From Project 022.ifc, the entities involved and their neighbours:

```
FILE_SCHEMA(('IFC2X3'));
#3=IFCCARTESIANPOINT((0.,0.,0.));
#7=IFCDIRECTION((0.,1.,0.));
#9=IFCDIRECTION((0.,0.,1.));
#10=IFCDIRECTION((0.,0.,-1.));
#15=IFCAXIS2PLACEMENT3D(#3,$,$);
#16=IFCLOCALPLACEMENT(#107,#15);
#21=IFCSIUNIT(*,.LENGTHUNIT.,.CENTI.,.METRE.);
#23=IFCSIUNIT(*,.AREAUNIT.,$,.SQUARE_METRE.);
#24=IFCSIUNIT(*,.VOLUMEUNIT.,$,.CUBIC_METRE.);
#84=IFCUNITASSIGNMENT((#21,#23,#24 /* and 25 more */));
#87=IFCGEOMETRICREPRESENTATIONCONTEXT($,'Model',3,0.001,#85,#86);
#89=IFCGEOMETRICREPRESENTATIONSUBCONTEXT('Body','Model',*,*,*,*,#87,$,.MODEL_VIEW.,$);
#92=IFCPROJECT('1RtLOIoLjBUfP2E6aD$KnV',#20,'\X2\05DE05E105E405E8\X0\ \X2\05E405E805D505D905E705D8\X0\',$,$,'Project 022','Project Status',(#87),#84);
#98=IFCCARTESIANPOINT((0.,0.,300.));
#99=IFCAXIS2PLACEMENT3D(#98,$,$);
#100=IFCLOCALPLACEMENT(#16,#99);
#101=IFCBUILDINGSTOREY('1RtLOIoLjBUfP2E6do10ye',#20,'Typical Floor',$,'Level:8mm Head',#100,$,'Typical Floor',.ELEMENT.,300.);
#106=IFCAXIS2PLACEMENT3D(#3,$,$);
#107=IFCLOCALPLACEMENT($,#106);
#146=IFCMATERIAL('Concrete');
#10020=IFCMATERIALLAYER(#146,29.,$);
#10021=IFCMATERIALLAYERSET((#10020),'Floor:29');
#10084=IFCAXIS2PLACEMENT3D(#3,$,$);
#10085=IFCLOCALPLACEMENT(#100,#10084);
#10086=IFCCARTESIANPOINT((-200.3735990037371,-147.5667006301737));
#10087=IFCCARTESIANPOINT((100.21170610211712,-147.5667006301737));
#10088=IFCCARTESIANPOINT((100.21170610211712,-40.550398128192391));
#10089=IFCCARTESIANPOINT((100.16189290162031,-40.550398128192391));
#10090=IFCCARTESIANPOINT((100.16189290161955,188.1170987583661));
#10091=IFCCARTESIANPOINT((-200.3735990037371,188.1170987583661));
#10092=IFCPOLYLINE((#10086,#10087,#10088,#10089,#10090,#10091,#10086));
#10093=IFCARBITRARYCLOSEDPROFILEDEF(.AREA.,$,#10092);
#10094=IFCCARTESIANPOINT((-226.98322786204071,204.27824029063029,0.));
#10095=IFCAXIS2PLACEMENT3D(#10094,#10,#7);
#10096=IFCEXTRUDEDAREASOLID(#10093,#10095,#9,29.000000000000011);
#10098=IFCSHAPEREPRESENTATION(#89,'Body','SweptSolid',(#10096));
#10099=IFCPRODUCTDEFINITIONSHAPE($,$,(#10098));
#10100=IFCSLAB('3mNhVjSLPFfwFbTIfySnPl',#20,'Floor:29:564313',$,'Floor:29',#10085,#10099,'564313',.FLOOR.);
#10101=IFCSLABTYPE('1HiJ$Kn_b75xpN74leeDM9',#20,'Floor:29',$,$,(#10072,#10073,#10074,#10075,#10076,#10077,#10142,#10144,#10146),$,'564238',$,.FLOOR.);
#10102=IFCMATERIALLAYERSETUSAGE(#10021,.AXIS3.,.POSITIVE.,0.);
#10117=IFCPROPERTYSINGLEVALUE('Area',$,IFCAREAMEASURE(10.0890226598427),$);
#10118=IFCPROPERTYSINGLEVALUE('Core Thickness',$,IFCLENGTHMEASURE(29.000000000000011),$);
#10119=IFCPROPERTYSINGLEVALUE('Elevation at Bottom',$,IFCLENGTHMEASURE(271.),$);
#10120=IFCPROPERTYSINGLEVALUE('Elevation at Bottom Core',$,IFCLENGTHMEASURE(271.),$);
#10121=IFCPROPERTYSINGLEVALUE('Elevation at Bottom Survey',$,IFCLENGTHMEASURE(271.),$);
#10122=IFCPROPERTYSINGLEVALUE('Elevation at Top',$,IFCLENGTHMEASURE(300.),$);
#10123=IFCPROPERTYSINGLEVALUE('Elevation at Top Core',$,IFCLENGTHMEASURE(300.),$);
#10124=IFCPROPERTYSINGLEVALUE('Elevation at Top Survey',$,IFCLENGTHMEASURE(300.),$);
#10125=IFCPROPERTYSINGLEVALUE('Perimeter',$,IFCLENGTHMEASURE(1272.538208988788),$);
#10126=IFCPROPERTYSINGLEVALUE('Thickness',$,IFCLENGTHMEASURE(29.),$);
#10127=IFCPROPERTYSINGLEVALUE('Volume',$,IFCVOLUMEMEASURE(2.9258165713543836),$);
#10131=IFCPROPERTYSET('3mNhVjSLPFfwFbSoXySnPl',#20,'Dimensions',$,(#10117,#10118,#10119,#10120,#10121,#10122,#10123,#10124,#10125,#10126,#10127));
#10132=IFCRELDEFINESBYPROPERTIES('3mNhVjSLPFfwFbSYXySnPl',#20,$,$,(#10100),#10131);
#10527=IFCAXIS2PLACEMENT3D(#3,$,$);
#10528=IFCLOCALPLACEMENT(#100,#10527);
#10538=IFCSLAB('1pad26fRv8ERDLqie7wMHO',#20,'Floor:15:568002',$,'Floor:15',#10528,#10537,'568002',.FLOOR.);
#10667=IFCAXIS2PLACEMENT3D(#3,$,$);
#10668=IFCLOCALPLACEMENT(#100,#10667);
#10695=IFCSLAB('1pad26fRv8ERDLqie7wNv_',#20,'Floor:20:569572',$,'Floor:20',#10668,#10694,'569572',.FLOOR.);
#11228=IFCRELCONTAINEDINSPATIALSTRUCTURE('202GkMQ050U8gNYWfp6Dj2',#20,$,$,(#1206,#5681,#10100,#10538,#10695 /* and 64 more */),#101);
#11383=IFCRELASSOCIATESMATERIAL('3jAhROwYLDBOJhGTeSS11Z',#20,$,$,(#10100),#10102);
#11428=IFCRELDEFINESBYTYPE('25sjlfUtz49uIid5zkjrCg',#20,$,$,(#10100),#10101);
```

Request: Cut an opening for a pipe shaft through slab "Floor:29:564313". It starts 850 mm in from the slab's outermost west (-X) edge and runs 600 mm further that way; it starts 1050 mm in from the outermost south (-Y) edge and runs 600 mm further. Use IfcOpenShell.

```python
import numpy as np
import ifcopenshell
import ifcopenshell.api.feature
import ifcopenshell.api.geometry
import ifcopenshell.api.pset
import ifcopenshell.api.root
import ifcopenshell.geom
import ifcopenshell.util.element
import ifcopenshell.util.placement
import ifcopenshell.util.representation
import ifcopenshell.util.shape
import ifcopenshell.util.unit

model = ifcopenshell.open("Project 022.ifc")
unit_scale = ifcopenshell.util.unit.calculate_unit_scale(model)
area_scale = ifcopenshell.util.unit.calculate_unit_scale(model, "AREAUNIT")
volume_scale = ifcopenshell.util.unit.calculate_unit_scale(model, "VOLUMEUNIT")
settings = ifcopenshell.geom.settings()


def volume(element):
    """Net volume in cubic metres, openings subtracted."""
    shape = ifcopenshell.geom.create_shape(settings, element)
    return ifcopenshell.util.shape.get_volume(shape.geometry)


slab = model.by_guid("3mNhVjSLPFfwFbTIfySnPl")
before = volume(slab)

# Extent in the slab's own axes, in metres. The edges named are its -X and -Y sides.
slab_shape = ifcopenshell.geom.create_shape(settings, slab)
vertices = ifcopenshell.util.shape.get_vertices(slab_shape.geometry)
x_min, y_min, bottom = vertices.min(axis=0)
top = vertices[:, 2].max()

opening = ifcopenshell.api.root.create_entity(model, ifc_class="IfcOpeningElement", name="Pipe shaft opening")
context = ifcopenshell.util.representation.get_context(model, "Model", "Body", "MODEL_VIEW")
width, depth = 0.6, 0.6
outline = [(0.0, 0.0), (width, 0.0), (width, depth), (0.0, depth), (0.0, 0.0)]
# Overshoot both faces by 50 mm so the cut is clean.
shape = ifcopenshell.api.geometry.add_slab_representation(
    model, context=context, depth=top - bottom + 0.1, polyline=outline
)
ifcopenshell.api.geometry.assign_representation(model, product=opening, representation=shape)

matrix = ifcopenshell.util.placement.get_local_placement(slab.ObjectPlacement)
matrix[:, 3] = matrix @ np.append(np.array([x_min + 0.85, y_min + 1.05, bottom - 0.05]) / unit_scale, 1.0)
ifcopenshell.api.geometry.edit_object_placement(model, product=opening, matrix=matrix, is_si=False)
ifcopenshell.api.feature.add_feature(model, feature=opening, element=slab)

after = volume(slab)

# Update the slab's stored quantities.
pset = model.by_id(ifcopenshell.util.element.get_pset(slab, "Dimensions", should_inherit=False)["id"])
ifcopenshell.api.pset.edit_pset(model, pset=pset, properties={
    "Area": model.create_entity("IfcAreaMeasure", after / (top - bottom) / area_scale),
    "Volume": model.create_entity("IfcVolumeMeasure", after / volume_scale),
})

print(f"slab volume {before:.3f} -> {after:.3f} m3")

model.write("Project 022-out.ifc")
```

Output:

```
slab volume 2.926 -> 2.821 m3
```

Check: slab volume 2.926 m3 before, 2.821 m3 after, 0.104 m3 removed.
